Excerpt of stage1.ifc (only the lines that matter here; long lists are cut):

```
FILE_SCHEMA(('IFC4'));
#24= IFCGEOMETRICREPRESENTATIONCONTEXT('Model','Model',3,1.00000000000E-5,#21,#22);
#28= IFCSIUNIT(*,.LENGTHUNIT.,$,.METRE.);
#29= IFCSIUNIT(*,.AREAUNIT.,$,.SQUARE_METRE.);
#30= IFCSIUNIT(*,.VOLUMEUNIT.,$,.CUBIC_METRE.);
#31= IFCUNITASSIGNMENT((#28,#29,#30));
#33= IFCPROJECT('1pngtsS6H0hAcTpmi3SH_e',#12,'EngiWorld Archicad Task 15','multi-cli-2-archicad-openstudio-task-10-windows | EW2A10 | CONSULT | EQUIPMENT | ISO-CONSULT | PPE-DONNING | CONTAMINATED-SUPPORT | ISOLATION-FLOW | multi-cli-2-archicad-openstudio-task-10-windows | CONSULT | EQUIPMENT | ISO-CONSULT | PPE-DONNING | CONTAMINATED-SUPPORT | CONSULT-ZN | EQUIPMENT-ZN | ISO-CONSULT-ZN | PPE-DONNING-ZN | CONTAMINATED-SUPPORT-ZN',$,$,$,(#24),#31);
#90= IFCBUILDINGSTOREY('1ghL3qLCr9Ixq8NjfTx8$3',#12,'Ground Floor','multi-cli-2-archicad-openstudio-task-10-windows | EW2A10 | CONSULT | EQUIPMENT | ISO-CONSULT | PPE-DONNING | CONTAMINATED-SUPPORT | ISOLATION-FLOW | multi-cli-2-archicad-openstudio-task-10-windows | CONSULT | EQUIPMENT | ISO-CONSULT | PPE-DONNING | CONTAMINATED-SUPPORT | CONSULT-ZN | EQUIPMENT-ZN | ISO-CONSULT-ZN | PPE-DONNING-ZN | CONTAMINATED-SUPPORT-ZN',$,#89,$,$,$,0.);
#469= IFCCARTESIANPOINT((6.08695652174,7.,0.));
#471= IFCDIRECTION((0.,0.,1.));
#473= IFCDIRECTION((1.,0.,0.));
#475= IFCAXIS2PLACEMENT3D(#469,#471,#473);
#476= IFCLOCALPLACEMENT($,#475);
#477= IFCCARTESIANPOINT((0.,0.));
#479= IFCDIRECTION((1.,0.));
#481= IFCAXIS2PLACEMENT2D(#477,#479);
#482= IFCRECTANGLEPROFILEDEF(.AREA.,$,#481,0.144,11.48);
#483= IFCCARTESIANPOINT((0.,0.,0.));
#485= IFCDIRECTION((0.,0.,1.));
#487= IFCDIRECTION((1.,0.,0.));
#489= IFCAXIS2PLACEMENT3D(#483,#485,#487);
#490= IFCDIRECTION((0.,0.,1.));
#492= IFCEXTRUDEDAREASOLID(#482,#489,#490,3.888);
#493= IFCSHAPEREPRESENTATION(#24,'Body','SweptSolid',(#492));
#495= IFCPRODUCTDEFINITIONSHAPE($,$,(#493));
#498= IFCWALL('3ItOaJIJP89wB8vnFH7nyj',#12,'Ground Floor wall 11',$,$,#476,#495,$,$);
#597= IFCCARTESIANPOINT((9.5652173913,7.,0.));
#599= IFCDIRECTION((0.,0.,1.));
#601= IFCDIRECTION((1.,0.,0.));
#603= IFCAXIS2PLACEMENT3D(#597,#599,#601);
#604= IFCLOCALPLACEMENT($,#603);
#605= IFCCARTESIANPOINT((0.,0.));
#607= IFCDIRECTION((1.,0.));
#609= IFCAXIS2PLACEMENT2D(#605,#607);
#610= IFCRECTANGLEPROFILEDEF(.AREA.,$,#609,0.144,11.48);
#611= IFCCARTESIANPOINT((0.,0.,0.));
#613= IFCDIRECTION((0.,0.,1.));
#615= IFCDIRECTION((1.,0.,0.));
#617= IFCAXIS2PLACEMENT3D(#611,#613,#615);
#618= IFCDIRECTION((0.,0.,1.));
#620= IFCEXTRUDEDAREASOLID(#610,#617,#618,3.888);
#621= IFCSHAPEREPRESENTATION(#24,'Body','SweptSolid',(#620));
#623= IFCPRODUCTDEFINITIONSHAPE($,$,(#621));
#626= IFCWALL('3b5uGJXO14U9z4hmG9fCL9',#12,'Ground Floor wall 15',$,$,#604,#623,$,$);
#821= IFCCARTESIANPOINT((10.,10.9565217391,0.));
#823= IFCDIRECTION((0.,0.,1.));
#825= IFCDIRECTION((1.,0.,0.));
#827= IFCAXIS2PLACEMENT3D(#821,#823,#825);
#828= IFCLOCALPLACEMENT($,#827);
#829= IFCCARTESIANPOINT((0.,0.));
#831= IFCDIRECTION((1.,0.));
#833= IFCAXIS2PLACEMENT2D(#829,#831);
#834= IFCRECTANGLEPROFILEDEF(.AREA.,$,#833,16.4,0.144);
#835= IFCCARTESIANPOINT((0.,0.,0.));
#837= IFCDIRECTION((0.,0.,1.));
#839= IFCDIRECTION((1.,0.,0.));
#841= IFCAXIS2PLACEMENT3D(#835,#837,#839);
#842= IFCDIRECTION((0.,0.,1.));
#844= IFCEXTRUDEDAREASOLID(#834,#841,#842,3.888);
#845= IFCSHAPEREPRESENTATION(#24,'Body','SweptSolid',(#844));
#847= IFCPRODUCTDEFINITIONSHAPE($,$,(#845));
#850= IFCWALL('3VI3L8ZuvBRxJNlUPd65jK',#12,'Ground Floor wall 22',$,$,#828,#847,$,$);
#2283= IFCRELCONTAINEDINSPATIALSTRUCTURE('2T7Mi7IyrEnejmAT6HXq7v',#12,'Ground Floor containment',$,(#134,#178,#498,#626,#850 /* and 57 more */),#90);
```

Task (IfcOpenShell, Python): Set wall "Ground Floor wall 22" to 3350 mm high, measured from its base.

```python
import ifcopenshell
import ifcopenshell.geom
import ifcopenshell.util.shape

model = ifcopenshell.open("stage1.ifc")
settings = ifcopenshell.geom.settings()


def volume(element):
    """Net volume in cubic metres, openings subtracted."""
    shape = ifcopenshell.geom.create_shape(settings, element)
    return ifcopenshell.util.shape.get_volume(shape.geometry)


wall = model.by_id(850)
before = volume(wall)

body = next(r for r in wall.Representation.Representations if r.RepresentationIdentifier == "Body")
solid = body.Items[0]
old_height = solid.Depth
solid.Depth = 3.35
after = volume(wall)

print(f"height {old_height:g} -> {solid.Depth:g}, volume {before:.3f} -> {after:.3f} m3")

model.write("stage1-out.ifc")
```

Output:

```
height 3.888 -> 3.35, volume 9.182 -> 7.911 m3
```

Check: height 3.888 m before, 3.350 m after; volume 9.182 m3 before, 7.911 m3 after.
